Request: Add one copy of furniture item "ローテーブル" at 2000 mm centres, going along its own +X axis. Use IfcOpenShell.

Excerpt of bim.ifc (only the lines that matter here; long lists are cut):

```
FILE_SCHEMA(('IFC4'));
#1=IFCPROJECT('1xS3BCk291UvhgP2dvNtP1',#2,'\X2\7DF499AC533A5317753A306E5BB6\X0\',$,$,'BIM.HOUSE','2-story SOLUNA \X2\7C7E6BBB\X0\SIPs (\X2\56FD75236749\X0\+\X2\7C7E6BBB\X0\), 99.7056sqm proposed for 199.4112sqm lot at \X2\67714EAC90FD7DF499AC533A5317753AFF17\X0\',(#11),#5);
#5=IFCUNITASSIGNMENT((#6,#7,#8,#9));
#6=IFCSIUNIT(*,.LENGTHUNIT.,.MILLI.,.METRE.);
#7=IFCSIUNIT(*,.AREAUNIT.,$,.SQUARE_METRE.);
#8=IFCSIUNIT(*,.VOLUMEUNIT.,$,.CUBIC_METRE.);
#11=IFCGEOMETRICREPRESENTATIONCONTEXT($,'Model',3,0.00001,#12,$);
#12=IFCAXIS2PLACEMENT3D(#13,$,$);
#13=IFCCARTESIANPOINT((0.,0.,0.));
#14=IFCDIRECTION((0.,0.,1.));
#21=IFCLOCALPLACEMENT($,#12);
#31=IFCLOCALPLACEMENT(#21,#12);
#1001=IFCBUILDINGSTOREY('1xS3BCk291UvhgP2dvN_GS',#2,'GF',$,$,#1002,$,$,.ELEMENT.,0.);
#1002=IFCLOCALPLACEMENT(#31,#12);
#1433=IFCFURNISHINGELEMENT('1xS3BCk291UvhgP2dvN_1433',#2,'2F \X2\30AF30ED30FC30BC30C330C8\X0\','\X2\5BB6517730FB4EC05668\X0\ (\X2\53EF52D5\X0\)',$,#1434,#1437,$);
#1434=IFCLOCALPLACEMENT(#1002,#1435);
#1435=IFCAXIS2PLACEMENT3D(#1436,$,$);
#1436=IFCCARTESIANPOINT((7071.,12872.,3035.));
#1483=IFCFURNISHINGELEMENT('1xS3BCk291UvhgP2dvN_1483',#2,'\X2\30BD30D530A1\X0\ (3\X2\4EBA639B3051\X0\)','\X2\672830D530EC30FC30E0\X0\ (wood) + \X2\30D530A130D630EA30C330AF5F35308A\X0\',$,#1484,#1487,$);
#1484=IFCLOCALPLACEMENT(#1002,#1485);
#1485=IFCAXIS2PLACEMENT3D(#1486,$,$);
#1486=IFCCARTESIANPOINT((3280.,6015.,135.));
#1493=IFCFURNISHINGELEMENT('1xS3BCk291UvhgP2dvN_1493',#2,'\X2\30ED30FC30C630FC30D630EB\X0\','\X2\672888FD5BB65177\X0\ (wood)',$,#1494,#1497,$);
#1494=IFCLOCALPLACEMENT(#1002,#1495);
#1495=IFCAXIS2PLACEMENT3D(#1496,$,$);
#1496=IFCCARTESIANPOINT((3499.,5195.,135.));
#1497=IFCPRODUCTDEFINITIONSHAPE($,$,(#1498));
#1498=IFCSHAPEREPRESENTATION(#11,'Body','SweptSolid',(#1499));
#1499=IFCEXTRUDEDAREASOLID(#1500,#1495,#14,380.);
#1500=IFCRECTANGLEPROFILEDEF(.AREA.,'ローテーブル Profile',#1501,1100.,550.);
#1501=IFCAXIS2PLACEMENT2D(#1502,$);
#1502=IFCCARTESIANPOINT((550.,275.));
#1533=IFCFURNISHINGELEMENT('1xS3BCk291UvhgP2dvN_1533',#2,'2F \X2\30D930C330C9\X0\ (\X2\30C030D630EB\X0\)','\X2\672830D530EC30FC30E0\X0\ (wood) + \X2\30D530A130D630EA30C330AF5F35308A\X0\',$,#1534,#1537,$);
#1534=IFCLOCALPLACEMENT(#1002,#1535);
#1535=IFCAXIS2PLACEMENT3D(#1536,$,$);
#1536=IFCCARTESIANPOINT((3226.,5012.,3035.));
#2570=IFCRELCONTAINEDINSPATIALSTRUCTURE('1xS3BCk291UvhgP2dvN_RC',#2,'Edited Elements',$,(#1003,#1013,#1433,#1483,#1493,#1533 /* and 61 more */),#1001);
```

```python
import ifcopenshell
import ifcopenshell.api.geometry
import ifcopenshell.api.root
import ifcopenshell.util.element
import ifcopenshell.util.placement
import ifcopenshell.util.unit

model = ifcopenshell.open("bim.ifc")
unit_scale = ifcopenshell.util.unit.calculate_unit_scale(model)


def reuse_history(source, copy):
    """copy_class also copies each property set's owner history, people and application; keep the originals."""
    for rel in copy.IsDefinedBy:
        if rel.is_a("IfcRelDefinesByProperties") and (history := rel.RelatingPropertyDefinition.OwnerHistory):
            rel.RelatingPropertyDefinition.OwnerHistory = source.OwnerHistory
            ifcopenshell.util.element.remove_deep2(model, history)


source = model.by_guid("1xS3BCk291UvhgP2dvN_1493")
base = ifcopenshell.util.placement.get_local_placement(source.ObjectPlacement)
step = base[:3, 0] * 2 / unit_scale

for i in range(1, 2):
    copy = ifcopenshell.api.root.copy_class(model, product=source)
    copy.Representation = ifcopenshell.util.element.copy_deep(
        model, source.Representation, exclude=["IfcGeometricRepresentationContext", "IfcRepresentationMap"]
    )
    reuse_history(source, copy)
    matrix = base.copy()
    matrix[:3, 3] += i * step
    print("added at", matrix[:3, 3].round(3) + 0.0)
    ifcopenshell.api.geometry.edit_object_placement(model, product=copy, matrix=matrix, is_si=False)

model.write("bim-out.ifc")
```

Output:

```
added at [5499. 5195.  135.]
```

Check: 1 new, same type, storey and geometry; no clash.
